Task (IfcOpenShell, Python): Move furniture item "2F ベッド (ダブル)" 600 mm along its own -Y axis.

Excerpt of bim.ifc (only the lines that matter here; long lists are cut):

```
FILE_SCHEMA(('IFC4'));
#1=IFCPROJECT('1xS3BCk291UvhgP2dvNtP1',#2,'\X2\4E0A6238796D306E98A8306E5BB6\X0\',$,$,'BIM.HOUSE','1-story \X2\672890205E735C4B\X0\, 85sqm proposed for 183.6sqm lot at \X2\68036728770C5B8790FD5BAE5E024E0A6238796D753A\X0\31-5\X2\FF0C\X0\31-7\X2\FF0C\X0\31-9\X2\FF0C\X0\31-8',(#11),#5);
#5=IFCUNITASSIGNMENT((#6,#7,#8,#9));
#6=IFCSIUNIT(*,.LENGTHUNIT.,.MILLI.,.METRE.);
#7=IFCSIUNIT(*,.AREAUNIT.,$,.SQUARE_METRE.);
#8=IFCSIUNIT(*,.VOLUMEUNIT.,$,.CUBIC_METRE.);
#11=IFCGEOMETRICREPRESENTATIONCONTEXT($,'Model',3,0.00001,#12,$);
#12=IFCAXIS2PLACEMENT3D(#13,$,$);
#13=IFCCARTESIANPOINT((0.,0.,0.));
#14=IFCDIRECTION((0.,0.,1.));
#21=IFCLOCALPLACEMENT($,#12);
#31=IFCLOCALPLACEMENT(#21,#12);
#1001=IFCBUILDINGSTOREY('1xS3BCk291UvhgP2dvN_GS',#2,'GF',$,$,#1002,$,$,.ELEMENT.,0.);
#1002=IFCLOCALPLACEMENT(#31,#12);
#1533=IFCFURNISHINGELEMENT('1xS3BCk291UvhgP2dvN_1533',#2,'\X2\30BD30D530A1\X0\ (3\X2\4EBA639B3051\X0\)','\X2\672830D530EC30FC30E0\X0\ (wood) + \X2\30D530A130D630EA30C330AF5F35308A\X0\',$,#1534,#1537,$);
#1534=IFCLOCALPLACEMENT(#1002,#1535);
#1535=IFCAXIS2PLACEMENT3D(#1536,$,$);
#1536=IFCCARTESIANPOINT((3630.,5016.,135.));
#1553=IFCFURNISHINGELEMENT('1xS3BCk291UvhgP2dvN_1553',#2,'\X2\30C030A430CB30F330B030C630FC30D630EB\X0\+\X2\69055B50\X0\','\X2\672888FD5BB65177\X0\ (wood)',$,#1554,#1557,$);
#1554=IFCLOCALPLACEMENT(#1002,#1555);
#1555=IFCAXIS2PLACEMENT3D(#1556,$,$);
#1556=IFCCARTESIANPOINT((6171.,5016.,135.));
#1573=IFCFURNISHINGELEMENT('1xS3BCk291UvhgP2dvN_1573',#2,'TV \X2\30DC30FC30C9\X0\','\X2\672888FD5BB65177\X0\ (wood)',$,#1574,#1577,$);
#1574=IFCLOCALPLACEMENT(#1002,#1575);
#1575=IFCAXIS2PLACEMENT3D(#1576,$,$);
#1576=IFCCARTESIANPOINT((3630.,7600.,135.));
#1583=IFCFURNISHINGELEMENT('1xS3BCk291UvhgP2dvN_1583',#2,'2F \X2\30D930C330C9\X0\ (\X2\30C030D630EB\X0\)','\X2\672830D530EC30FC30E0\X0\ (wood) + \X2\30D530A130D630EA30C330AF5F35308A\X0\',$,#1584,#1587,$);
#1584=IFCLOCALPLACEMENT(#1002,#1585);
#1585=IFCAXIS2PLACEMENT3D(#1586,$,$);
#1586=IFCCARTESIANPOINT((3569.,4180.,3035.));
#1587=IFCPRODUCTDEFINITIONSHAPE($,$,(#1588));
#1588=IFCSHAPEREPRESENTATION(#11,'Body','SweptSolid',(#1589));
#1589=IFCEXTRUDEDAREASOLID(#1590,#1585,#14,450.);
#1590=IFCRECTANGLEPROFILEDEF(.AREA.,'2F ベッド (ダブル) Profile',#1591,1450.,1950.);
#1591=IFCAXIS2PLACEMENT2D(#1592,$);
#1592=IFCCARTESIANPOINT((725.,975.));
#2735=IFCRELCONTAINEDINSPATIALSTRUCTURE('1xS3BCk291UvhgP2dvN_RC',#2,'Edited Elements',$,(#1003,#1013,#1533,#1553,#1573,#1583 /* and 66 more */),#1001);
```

```python
import ifcopenshell
import ifcopenshell.api.geometry
import ifcopenshell.util.placement
import ifcopenshell.util.unit

model = ifcopenshell.open("bim.ifc")
unit_scale = ifcopenshell.util.unit.calculate_unit_scale(model)

item = model.by_guid("1xS3BCk291UvhgP2dvN_1583")
matrix = ifcopenshell.util.placement.get_local_placement(item.ObjectPlacement)
matrix[:3, 3] -= matrix[:3, 1] * 0.6 / unit_scale
ifcopenshell.api.geometry.edit_object_placement(model, product=item, matrix=matrix, is_si=False)

print(ifcopenshell.util.placement.get_local_placement(item.ObjectPlacement).round(3) + 0.0)

model.write("bim_v2.ifc")
```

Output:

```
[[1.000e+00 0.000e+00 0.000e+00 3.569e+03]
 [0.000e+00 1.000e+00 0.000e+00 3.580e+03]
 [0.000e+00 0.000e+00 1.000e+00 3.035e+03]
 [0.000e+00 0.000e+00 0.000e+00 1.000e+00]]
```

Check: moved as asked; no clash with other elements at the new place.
